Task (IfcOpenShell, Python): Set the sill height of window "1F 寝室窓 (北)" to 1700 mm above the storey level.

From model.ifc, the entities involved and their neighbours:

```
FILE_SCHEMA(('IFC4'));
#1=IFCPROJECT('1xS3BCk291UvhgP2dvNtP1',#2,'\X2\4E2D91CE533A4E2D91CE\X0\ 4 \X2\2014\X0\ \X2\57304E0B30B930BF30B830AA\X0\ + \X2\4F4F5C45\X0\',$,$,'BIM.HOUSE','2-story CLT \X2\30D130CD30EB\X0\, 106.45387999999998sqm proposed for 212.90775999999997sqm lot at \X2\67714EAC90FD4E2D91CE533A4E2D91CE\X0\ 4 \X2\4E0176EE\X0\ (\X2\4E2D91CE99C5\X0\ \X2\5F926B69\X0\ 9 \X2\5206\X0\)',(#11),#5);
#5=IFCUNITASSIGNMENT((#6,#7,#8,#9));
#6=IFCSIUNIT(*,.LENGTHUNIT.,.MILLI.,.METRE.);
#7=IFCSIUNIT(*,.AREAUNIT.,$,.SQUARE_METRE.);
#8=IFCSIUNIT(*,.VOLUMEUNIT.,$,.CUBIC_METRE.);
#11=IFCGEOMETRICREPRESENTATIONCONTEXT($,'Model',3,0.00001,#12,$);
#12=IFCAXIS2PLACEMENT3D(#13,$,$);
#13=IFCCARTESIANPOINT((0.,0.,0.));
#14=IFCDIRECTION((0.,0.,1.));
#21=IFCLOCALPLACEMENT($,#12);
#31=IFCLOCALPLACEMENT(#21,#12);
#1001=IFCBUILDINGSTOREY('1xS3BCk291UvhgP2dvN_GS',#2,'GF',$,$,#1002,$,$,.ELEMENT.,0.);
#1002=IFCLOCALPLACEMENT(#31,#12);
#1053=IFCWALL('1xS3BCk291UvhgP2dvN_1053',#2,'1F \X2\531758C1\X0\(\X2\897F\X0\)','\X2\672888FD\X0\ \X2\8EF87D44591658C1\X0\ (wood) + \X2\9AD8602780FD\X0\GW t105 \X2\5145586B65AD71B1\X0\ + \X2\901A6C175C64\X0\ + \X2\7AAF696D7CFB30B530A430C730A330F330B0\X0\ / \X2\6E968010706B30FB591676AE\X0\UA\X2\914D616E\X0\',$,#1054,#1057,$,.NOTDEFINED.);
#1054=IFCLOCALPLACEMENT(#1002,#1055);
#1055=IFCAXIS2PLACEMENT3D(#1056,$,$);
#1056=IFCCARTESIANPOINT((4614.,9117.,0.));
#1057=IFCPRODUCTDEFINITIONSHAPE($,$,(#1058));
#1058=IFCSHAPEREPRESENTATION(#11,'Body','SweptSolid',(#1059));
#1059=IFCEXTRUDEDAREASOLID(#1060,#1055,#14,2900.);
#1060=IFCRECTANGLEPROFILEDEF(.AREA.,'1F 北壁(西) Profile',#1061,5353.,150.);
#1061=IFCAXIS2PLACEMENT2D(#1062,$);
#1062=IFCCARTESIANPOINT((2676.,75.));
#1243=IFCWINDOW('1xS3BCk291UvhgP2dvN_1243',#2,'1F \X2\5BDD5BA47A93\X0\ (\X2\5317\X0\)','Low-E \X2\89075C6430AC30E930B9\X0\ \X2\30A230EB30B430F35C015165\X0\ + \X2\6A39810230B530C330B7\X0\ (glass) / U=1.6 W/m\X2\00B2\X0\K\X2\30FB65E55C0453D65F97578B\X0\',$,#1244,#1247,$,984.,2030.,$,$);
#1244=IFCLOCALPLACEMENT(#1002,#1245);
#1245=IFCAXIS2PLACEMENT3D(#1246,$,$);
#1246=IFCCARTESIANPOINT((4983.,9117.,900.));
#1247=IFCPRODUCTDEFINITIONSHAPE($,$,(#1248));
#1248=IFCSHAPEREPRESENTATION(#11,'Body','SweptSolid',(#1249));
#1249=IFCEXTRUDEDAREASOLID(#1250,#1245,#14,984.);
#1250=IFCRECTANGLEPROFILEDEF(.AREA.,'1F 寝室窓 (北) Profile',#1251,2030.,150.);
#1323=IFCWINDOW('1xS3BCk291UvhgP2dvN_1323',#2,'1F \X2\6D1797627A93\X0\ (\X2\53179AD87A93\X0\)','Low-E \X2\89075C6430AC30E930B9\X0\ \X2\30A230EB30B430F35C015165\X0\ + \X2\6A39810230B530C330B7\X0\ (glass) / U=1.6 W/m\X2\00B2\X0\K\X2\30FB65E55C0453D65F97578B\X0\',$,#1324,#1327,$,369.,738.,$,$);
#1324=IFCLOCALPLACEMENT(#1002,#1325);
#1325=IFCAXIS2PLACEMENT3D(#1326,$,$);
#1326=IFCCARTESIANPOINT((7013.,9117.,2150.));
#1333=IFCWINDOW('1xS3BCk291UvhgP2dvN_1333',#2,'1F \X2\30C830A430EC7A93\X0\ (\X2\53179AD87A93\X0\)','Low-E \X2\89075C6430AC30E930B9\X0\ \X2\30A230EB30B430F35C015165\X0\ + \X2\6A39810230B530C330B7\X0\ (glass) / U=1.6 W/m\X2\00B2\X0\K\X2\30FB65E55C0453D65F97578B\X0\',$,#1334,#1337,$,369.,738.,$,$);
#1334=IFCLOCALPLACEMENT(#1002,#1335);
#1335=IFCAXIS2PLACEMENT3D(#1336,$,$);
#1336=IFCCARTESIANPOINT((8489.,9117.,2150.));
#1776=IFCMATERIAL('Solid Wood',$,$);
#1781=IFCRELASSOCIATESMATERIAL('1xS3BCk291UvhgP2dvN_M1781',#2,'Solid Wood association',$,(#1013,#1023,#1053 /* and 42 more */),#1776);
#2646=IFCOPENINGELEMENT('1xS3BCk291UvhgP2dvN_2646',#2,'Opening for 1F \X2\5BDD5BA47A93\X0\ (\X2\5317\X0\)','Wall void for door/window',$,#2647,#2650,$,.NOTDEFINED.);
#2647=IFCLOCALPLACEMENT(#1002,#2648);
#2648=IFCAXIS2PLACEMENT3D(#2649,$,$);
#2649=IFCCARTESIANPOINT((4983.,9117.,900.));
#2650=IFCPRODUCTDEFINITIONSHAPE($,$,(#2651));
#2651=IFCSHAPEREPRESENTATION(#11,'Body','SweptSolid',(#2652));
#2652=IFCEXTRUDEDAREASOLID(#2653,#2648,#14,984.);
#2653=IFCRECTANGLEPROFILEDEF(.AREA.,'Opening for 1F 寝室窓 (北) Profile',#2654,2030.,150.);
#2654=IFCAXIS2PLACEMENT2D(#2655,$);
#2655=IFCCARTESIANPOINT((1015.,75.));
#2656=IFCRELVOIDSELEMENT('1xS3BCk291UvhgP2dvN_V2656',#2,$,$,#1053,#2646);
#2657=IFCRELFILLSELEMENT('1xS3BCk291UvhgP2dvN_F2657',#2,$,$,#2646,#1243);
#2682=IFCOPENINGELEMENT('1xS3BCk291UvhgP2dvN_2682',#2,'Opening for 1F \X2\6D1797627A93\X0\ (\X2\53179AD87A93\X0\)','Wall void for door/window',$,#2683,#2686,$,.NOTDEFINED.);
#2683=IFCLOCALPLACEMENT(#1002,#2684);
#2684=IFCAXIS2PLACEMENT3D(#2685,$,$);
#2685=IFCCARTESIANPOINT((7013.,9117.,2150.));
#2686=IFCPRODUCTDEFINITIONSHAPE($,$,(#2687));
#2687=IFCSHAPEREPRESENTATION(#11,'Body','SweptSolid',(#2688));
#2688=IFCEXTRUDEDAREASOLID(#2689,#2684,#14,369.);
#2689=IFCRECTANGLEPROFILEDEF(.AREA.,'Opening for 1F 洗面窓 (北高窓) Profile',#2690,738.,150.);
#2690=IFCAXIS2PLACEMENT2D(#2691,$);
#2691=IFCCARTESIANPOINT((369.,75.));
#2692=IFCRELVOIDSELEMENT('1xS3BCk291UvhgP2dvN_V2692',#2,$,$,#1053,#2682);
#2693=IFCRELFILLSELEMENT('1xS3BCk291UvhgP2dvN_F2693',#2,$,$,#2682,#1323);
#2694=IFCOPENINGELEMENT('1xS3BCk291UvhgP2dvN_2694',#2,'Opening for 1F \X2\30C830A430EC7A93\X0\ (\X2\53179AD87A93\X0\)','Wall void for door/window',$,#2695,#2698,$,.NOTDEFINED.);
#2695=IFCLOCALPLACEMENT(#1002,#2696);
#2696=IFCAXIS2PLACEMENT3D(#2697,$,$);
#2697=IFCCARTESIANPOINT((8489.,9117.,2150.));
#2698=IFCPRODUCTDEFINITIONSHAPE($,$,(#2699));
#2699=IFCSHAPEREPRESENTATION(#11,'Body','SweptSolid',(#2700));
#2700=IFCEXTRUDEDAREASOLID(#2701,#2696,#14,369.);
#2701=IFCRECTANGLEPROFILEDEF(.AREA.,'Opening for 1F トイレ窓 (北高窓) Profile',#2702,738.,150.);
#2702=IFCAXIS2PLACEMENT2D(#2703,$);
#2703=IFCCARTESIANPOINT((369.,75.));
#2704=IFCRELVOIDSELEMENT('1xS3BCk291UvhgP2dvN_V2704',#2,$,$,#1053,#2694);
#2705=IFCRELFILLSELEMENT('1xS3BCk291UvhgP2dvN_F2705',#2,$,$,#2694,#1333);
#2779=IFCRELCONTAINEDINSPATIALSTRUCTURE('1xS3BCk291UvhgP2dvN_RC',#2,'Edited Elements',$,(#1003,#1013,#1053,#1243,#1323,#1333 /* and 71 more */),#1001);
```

```python
import numpy as np
import ifcopenshell
import ifcopenshell.api.geometry
import ifcopenshell.geom
import ifcopenshell.util.element
import ifcopenshell.util.placement
import ifcopenshell.util.shape
import ifcopenshell.util.unit

model = ifcopenshell.open("model.ifc")
unit_scale = ifcopenshell.util.unit.calculate_unit_scale(model)

window = model.by_id(1243)
opening = window.FillsVoids[0].RelatingOpeningElement
storey = ifcopenshell.util.element.get_container(window, ifc_class="IfcBuildingStorey")
level = ifcopenshell.util.placement.get_local_placement(storey.ObjectPlacement)[2, 3]

# The opening's origin need not be at the sill, so measure its lowest point.
shape = ifcopenshell.geom.create_shape(ifcopenshell.geom.settings(), opening)
bottom = ifcopenshell.util.shape.get_shape_bottom_elevation(shape, shape.geometry) / unit_scale
dz = level + 1700.0 - bottom

shift = np.array([0.0, 0.0, dz])
# The window is not placed relative to its opening, so move both.
for product in (opening, window):
    matrix = ifcopenshell.util.placement.get_local_placement(product.ObjectPlacement)
    matrix[:3, 3] += shift
    ifcopenshell.api.geometry.edit_object_placement(model, product=product, matrix=matrix, is_si=False)

print(f"moved by {dz * unit_scale:+.3f} m")

model.write("model-out.ifc")
```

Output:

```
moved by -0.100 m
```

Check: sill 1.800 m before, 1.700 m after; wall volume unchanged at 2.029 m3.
